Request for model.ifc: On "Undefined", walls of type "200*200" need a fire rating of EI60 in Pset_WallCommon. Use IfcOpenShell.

First a look at what the model holds.

```python
import ifcopenshell
import ifcopenshell.util.element

model = ifcopenshell.open("model.ifc")
print(model.schema)
storey = next(s for s in model.by_type("IfcBuildingStorey") if s.Name == "Undefined")
walls = [e for e in ifcopenshell.util.element.get_decomposition(storey) if e.is_a("IfcWall")]
seen = {}
for e in walls:
    element_type = ifcopenshell.util.element.get_type(e)
    key = (element_type.Name if element_type != e and element_type else None, ifcopenshell.util.element.get_pset(e, "Pset_WallCommon", "FireRating"))
    seen[key] = seen.get(key, 0) + 1
for (name, value), count in sorted(seen.items(), key=str):
    print(count, "x", name, "|", value)
```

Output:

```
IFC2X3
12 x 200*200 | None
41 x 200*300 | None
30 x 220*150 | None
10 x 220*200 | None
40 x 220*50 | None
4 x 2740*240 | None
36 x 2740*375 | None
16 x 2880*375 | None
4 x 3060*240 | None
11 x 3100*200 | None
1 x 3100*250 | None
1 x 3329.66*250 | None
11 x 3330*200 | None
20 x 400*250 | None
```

```python
import ifcopenshell
import ifcopenshell.api.pset
import ifcopenshell.util.element

model = ifcopenshell.open("model.ifc")

storey = next(s for s in model.by_type("IfcBuildingStorey") if s.Name == "Undefined")
walls = [e for e in ifcopenshell.util.element.get_decomposition(storey) if e.is_a("IfcWall")]

count = 0
for e in walls:
    element_type = ifcopenshell.util.element.get_type(e)
    if element_type in (None, e) or element_type.Name != "200*200":
        continue
    # add_pset returns the element's existing set when there is one.
    pset = ifcopenshell.api.pset.add_pset(model, product=e, name="Pset_WallCommon")
    ifcopenshell.api.pset.edit_pset(model, pset=pset, properties={"FireRating": "EI60"})
    count += 1

print(count, "walls updated")

model.write("model_v2.ifc")
```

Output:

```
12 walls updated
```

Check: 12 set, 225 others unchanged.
